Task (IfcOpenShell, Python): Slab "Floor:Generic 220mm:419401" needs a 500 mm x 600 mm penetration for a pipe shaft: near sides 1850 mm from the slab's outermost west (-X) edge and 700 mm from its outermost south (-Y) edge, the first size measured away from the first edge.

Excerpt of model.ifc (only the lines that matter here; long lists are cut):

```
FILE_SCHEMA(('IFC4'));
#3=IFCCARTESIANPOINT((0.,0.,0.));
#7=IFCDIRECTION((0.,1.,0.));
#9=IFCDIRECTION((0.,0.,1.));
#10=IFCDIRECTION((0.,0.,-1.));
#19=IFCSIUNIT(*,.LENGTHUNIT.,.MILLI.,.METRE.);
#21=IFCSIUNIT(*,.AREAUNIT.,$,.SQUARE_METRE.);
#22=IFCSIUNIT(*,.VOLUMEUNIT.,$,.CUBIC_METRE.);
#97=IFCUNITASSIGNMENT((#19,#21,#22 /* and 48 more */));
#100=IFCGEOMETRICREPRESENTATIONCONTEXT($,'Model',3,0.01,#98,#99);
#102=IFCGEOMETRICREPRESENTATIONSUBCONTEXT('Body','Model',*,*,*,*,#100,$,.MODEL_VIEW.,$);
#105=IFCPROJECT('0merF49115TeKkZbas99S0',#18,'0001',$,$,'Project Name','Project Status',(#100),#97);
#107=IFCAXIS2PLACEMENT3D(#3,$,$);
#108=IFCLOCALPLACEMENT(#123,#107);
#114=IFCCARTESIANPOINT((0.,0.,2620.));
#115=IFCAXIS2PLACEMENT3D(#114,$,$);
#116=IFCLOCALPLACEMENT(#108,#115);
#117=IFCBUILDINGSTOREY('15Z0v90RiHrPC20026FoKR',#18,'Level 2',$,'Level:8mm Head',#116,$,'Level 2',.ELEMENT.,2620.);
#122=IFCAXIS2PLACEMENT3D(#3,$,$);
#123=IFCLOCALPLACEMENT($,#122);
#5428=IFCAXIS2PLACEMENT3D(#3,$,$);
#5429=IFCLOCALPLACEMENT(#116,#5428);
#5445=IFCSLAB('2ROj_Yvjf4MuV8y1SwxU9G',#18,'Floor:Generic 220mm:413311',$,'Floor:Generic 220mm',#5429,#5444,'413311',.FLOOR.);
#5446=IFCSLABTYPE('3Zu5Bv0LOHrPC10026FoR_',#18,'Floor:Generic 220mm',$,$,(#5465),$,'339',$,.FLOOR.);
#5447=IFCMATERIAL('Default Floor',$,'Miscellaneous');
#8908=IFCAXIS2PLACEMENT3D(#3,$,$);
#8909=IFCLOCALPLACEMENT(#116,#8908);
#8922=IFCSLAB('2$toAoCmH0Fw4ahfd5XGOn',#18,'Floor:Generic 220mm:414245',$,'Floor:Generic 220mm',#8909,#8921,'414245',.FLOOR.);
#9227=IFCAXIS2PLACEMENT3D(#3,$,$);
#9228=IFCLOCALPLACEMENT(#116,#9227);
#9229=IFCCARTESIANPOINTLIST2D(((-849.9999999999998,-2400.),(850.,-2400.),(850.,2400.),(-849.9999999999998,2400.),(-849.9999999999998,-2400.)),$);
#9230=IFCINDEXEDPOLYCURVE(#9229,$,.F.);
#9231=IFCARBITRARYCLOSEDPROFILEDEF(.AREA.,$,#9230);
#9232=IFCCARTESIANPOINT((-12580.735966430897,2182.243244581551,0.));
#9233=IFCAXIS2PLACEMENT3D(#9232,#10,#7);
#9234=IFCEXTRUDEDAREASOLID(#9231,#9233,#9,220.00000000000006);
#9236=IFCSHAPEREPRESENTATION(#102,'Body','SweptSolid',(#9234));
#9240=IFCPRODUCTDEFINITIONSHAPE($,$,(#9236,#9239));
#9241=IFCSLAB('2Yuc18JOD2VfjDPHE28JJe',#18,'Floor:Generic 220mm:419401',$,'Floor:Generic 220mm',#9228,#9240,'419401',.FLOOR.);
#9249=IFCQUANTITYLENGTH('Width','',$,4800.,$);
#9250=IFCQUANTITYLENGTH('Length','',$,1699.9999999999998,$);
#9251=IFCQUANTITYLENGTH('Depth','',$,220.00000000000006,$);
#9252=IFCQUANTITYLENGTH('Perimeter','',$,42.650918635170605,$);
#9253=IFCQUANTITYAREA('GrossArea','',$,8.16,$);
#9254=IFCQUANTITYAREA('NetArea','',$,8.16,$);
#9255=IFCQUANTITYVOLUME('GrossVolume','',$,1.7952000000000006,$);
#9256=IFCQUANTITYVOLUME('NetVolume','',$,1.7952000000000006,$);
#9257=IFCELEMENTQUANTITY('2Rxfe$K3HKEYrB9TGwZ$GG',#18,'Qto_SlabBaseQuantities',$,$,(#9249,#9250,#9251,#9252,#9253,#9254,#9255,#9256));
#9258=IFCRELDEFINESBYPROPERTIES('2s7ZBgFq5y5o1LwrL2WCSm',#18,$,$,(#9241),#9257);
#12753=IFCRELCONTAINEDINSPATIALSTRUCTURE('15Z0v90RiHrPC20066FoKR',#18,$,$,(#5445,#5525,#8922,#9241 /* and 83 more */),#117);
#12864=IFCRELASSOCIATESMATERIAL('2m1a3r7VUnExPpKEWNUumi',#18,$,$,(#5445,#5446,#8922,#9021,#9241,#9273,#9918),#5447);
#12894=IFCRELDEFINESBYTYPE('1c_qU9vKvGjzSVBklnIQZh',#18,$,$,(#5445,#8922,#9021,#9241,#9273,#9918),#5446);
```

```python
import numpy as np
import ifcopenshell
import ifcopenshell.api.feature
import ifcopenshell.api.geometry
import ifcopenshell.api.pset
import ifcopenshell.api.root
import ifcopenshell.geom
import ifcopenshell.util.element
import ifcopenshell.util.placement
import ifcopenshell.util.representation
import ifcopenshell.util.shape
import ifcopenshell.util.unit

model = ifcopenshell.open("model.ifc")
unit_scale = ifcopenshell.util.unit.calculate_unit_scale(model)
area_scale = ifcopenshell.util.unit.calculate_unit_scale(model, "AREAUNIT")
volume_scale = ifcopenshell.util.unit.calculate_unit_scale(model, "VOLUMEUNIT")
settings = ifcopenshell.geom.settings()


def volume(element):
    """Net volume in cubic metres, openings subtracted."""
    shape = ifcopenshell.geom.create_shape(settings, element)
    return ifcopenshell.util.shape.get_volume(shape.geometry)


slab = model.by_id(9241)
before = volume(slab)

# Extent in the slab's own axes, in metres. The edges named are its -X and -Y sides.
slab_shape = ifcopenshell.geom.create_shape(settings, slab)
vertices = ifcopenshell.util.shape.get_vertices(slab_shape.geometry)
x_min, y_min, bottom = vertices.min(axis=0)
top = vertices[:, 2].max()

opening = ifcopenshell.api.root.create_entity(model, ifc_class="IfcOpeningElement", name="Pipe shaft opening", predefined_type="OPENING")
context = ifcopenshell.util.representation.get_context(model, "Model", "Body", "MODEL_VIEW")
width, depth = 0.5, 0.6
outline = [(0.0, 0.0), (width, 0.0), (width, depth), (0.0, depth), (0.0, 0.0)]
# Overshoot both faces by 50 mm so the cut is clean.
shape = ifcopenshell.api.geometry.add_slab_representation(
    model, context=context, depth=top - bottom + 0.1, polyline=outline
)
ifcopenshell.api.geometry.assign_representation(model, product=opening, representation=shape)

matrix = ifcopenshell.util.placement.get_local_placement(slab.ObjectPlacement)
matrix[:, 3] = matrix @ np.append(np.array([x_min + 1.85, y_min + 0.7, bottom - 0.05]) / unit_scale, 1.0)
ifcopenshell.api.geometry.edit_object_placement(model, product=opening, matrix=matrix, is_si=False)
ifcopenshell.api.feature.add_feature(model, feature=opening, element=slab)

after = volume(slab)

# Update the slab's stored quantities.
qto = model.by_id(ifcopenshell.util.element.get_pset(slab, "Qto_SlabBaseQuantities", should_inherit=False)["id"])
ifcopenshell.api.pset.edit_qto(model, qto=qto, properties={
    "NetArea": after / (top - bottom) / area_scale,
    "NetVolume": after / volume_scale,
})

print(f"slab volume {before:.3f} -> {after:.3f} m3")

model.write("model_rev.ifc")
```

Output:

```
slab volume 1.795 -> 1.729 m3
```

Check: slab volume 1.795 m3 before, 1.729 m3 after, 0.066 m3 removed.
